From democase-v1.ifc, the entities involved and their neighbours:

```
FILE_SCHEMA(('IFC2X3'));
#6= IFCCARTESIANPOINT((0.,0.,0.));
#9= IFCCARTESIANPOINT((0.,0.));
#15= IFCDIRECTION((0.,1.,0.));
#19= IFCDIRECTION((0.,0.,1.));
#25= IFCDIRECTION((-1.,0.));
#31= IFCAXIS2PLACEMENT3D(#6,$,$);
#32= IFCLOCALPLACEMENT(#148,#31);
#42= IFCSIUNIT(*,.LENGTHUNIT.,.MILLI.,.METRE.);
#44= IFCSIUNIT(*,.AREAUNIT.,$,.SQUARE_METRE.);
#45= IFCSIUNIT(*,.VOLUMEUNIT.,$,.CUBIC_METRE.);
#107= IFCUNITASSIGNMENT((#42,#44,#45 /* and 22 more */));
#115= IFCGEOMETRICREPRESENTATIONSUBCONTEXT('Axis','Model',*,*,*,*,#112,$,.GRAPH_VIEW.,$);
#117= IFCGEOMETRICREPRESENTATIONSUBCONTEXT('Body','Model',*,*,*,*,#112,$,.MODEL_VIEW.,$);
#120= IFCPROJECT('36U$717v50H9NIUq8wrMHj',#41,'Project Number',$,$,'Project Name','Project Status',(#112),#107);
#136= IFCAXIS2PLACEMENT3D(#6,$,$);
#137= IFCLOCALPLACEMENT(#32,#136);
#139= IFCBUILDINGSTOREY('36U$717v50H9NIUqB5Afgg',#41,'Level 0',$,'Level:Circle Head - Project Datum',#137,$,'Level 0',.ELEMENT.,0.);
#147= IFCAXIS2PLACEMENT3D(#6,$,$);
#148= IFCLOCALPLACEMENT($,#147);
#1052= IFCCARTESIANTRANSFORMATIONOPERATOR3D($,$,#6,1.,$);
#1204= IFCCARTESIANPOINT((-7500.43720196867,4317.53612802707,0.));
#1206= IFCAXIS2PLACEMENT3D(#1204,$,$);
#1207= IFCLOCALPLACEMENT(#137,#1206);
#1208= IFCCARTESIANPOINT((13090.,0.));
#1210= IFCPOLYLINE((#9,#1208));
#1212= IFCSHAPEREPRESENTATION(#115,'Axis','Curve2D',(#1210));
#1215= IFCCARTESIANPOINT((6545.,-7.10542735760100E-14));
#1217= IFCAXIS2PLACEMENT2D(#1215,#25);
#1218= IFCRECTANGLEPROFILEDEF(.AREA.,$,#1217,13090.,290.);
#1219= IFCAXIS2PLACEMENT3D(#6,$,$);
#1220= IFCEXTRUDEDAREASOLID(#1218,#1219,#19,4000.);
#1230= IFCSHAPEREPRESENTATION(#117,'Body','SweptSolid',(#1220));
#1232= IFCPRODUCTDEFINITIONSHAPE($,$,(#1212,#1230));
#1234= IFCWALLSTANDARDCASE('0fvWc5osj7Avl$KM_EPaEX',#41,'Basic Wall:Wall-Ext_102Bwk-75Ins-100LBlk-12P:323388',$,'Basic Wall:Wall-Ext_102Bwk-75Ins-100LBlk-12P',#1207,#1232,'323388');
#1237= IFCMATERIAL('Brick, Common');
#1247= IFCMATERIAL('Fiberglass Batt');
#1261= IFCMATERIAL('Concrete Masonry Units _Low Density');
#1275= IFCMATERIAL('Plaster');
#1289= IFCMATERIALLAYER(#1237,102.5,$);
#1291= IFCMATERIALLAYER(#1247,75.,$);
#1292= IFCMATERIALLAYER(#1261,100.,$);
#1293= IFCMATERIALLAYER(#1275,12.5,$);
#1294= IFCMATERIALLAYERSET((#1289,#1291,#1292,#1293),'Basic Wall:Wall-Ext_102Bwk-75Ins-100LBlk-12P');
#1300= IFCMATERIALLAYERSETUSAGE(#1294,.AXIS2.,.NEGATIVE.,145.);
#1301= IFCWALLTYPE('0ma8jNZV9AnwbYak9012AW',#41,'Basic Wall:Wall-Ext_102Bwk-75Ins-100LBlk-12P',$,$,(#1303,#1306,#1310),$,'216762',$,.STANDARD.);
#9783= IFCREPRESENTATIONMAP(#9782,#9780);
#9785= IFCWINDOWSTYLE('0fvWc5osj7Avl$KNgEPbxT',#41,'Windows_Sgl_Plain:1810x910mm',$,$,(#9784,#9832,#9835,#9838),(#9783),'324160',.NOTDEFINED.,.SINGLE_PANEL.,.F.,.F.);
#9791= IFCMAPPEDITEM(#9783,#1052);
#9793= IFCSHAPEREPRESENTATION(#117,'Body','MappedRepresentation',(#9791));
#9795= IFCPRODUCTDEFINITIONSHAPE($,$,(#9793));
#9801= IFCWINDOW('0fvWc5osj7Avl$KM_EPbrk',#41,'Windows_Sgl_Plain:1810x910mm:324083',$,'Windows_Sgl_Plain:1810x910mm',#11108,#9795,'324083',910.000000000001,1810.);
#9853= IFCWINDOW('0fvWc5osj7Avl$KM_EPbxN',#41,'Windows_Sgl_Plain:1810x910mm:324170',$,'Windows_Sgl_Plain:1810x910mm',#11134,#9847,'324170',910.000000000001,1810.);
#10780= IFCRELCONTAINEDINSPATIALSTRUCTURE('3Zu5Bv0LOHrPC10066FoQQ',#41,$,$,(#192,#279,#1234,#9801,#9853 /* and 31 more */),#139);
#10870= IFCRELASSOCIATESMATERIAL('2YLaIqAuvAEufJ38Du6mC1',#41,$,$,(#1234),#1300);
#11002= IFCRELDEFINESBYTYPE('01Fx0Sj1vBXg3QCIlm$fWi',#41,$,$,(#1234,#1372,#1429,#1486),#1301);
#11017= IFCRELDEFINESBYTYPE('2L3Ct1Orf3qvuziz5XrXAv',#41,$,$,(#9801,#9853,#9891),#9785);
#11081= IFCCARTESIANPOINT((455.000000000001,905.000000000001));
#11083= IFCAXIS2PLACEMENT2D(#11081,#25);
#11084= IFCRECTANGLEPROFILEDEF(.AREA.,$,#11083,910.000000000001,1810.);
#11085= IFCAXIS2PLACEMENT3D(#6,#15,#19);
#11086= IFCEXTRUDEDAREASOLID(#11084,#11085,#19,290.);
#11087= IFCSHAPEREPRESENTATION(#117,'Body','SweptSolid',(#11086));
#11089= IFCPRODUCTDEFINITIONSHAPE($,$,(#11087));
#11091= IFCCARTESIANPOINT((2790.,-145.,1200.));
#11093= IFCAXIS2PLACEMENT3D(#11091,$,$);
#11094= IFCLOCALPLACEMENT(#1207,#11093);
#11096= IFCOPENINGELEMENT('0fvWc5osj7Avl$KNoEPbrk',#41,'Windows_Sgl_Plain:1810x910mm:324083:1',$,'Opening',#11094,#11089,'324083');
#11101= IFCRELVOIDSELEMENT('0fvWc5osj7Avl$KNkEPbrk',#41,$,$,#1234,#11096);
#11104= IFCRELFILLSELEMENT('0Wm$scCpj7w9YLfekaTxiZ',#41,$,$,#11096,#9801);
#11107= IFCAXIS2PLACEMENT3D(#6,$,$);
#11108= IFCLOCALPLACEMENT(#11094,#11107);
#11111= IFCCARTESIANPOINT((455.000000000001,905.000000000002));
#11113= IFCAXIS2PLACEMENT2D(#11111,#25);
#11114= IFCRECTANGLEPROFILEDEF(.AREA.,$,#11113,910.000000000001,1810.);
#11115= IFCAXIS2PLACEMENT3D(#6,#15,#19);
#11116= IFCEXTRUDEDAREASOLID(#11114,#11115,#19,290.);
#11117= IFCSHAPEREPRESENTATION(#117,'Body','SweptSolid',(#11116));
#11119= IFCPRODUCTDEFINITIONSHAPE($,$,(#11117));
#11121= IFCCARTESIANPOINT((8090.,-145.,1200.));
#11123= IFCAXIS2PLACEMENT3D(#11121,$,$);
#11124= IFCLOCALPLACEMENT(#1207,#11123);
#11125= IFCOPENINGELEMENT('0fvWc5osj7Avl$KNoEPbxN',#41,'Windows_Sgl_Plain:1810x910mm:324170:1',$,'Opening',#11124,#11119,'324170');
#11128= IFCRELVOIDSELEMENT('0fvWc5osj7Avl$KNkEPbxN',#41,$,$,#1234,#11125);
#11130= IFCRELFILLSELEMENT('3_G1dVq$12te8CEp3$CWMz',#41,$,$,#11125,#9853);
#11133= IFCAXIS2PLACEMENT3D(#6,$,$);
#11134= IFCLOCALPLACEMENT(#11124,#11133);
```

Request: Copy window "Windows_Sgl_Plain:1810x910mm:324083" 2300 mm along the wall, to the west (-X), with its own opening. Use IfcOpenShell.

```python
import ifcopenshell
import ifcopenshell.api.feature
import ifcopenshell.api.geometry
import ifcopenshell.api.root
import ifcopenshell.geom
import ifcopenshell.util.element
import ifcopenshell.util.placement
import ifcopenshell.util.shape
import ifcopenshell.util.unit

model = ifcopenshell.open("democase-v1.ifc")
unit_scale = ifcopenshell.util.unit.calculate_unit_scale(model)
settings = ifcopenshell.geom.settings()


def volume(element):
    """Net volume in cubic metres, openings subtracted."""
    shape = ifcopenshell.geom.create_shape(settings, element)
    return ifcopenshell.util.shape.get_volume(shape.geometry)


def reuse_history(source, copy):
    """copy_class also copies each property set's owner history, people and application; keep the originals."""
    for rel in copy.IsDefinedBy:
        if rel.is_a("IfcRelDefinesByProperties") and (history := rel.RelatingPropertyDefinition.OwnerHistory):
            rel.RelatingPropertyDefinition.OwnerHistory = source.OwnerHistory
            ifcopenshell.util.element.remove_deep2(model, history)


window = model.by_guid("0fvWc5osj7Avl$KM_EPbrk")
opening = window.FillsVoids[0].RelatingOpeningElement
wall = opening.VoidsElements[0].RelatingBuildingElement
before = volume(wall)
shift = ifcopenshell.util.placement.get_local_placement(wall.ObjectPlacement)[:3, 0] * -2.3 / unit_scale

# copy_class copies the void relationship, type, container and properties, but no geometry.
new_opening = ifcopenshell.api.root.copy_class(model, product=opening)
new_opening.Representation = ifcopenshell.util.element.copy_deep(
    model, opening.Representation, exclude=["IfcGeometricRepresentationContext", "IfcRepresentationMap"]
)
new_opening.Name = "Windows_Sgl_Plain:1810x910mm"
new_opening.Tag = None
new_window = ifcopenshell.api.root.copy_class(model, product=window)
new_window.Representation = ifcopenshell.util.element.copy_deep(
    model, window.Representation, exclude=["IfcGeometricRepresentationContext", "IfcRepresentationMap"]
)
new_window.Name = "Windows_Sgl_Plain:1810x910mm"
new_window.Tag = None
reuse_history(window, new_window)
fills = ifcopenshell.api.feature.add_filling(model, opening=new_opening, element=new_window)
fills.OwnerHistory = new_window.OwnerHistory  # required in IFC2X3

for old, new in ((opening, new_opening), (window, new_window)):
    matrix = ifcopenshell.util.placement.get_local_placement(old.ObjectPlacement)
    matrix[:3, 3] += shift
    ifcopenshell.api.geometry.edit_object_placement(model, product=new, matrix=matrix, is_si=False)

after = volume(wall)

print(f"wall volume {before:.3f} -> {after:.3f} m3")

model.write("democase-v1_updated.ifc")
```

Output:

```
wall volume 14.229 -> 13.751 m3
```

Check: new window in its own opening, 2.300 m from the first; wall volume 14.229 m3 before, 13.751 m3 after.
